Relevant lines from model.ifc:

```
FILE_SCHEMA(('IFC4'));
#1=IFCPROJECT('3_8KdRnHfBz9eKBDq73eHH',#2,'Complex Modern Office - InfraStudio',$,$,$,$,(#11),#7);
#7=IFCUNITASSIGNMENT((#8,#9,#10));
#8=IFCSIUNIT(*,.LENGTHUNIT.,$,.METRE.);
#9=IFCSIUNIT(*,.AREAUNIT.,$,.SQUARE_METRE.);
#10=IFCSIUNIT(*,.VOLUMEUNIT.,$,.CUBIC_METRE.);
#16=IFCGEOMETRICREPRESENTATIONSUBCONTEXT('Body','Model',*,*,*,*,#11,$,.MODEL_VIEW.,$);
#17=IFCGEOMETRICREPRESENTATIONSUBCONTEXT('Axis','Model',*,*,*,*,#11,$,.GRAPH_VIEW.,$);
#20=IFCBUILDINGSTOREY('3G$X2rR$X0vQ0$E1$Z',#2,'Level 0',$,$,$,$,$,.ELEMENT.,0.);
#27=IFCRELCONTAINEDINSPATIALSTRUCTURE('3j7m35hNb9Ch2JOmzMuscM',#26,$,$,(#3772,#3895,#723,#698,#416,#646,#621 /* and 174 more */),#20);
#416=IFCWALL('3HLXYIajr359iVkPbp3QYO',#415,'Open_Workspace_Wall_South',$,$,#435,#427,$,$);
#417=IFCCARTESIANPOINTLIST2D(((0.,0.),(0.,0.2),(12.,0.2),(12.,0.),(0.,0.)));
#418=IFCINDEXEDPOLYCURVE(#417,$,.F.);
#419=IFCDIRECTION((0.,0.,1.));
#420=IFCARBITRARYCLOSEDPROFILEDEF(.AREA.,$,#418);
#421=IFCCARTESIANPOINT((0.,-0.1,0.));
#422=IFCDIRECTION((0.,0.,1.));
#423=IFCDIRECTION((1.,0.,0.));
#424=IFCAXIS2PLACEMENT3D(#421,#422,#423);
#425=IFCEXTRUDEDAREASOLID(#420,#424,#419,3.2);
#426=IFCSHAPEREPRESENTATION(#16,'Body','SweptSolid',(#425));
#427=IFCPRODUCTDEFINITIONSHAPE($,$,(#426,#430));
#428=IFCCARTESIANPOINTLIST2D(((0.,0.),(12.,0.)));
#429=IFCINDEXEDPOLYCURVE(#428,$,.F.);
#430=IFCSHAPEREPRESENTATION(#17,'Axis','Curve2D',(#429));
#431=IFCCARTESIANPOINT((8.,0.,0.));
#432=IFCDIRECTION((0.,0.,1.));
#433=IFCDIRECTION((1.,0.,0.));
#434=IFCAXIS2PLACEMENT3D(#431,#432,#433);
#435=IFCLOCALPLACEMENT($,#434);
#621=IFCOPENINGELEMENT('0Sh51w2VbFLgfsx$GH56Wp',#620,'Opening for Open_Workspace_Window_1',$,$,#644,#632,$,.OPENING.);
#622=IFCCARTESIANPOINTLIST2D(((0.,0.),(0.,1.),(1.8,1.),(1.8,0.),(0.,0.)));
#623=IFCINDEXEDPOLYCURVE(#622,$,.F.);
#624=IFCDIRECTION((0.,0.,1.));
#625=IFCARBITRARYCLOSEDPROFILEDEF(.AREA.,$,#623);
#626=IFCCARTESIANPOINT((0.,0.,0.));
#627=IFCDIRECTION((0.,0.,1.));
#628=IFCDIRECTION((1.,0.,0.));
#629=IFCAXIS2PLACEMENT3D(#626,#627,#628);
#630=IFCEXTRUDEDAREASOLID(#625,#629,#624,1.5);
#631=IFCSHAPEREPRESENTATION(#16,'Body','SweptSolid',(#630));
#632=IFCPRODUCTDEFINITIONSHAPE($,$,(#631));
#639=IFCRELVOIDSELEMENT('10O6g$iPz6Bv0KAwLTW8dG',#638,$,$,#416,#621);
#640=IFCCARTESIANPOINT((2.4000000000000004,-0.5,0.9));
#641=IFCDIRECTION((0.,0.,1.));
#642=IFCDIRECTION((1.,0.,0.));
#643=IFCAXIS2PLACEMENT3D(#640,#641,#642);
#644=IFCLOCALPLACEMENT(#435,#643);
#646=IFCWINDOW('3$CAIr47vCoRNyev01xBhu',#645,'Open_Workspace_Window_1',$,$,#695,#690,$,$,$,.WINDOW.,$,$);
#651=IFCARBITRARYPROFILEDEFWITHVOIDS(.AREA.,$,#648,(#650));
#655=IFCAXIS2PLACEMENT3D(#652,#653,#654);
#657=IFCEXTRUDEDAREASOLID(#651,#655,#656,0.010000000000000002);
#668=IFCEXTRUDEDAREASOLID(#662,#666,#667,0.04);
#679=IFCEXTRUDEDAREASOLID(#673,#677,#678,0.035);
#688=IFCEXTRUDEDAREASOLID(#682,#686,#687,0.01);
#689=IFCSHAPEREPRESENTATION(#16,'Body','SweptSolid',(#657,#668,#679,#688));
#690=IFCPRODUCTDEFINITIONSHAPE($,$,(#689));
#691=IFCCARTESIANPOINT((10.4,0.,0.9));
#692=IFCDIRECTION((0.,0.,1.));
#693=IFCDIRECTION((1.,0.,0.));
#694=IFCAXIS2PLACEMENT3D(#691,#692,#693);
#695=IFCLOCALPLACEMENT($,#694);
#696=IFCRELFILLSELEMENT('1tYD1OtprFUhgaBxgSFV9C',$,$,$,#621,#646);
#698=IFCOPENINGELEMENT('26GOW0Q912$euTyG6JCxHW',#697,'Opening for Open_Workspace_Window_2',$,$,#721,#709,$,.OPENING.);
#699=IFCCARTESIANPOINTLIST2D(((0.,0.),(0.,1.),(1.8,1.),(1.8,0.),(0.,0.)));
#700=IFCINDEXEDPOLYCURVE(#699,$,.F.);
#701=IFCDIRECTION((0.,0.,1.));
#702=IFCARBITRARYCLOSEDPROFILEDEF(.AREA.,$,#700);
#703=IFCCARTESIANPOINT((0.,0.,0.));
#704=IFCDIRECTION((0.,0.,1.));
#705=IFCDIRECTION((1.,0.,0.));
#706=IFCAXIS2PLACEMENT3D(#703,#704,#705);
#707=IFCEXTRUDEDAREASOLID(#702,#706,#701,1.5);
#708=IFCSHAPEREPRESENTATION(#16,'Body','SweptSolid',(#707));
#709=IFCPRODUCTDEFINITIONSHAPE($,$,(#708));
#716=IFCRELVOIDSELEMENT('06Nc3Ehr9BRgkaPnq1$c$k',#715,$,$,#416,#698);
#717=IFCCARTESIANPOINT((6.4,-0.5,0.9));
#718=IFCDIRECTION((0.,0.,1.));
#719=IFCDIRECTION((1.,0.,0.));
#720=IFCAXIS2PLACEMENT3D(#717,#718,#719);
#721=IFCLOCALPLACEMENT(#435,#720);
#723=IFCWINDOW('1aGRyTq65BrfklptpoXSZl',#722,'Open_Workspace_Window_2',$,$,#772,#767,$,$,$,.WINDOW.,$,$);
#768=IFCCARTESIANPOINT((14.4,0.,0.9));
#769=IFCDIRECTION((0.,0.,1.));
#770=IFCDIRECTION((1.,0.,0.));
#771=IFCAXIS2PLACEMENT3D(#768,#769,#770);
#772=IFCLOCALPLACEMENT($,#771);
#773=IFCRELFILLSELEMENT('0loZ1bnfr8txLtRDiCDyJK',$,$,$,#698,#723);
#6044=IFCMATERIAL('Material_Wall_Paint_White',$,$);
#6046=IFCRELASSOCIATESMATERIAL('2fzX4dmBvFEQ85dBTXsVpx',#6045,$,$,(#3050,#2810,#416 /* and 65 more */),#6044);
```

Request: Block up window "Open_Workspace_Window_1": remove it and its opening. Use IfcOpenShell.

```python
import ifcopenshell
import ifcopenshell.api.feature
import ifcopenshell.api.root
import ifcopenshell.geom
import ifcopenshell.util.shape

model = ifcopenshell.open("model.ifc")
settings = ifcopenshell.geom.settings()


def volume(element):
    """Net volume in cubic metres, openings subtracted."""
    shape = ifcopenshell.geom.create_shape(settings, element)
    return ifcopenshell.util.shape.get_volume(shape.geometry)


window = model.by_guid("3$CAIr47vCoRNyev01xBhu")
opening = window.FillsVoids[0].RelatingOpeningElement
wall = opening.VoidsElements[0].RelatingBuildingElement
before = volume(wall)

ifcopenshell.api.root.remove_product(model, product=window)
ifcopenshell.api.feature.remove_feature(model, feature=opening)

after = volume(wall)

print(f"wall volume {before:.3f} -> {after:.3f} m3")

model.write("model_rev.ifc")
```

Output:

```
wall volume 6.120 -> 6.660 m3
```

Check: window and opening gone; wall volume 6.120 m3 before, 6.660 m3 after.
